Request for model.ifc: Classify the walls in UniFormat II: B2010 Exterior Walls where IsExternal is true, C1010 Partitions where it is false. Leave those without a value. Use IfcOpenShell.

First a look at what the model holds.

```python
import ifcopenshell
import ifcopenshell.util.element

model = ifcopenshell.open("model.ifc")
print(model.schema)
print("classifications:", [c.Name for c in model.by_type("IfcClassification")])
values = [ifcopenshell.util.element.get_pset(e, "Pset_WallCommon", "IsExternal") for e in model.by_type("IfcWall")]
for value in (True, False, None):
    print("IsExternal", value, values.count(value))
```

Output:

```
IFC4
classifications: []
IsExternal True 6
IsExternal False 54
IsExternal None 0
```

```python
import ifcopenshell
import ifcopenshell.api.classification
import ifcopenshell.util.element

model = ifcopenshell.open("model.ifc")

system = ifcopenshell.api.classification.add_classification(model, classification="UniFormat II")

walls = model.by_type("IfcWall")
external = {e: ifcopenshell.util.element.get_pset(e, "Pset_WallCommon", "IsExternal") for e in walls}
for flag, code, name in ((True, "B2010", "Exterior Walls"), (False, "C1010", "Partitions")):
    products = [e for e in walls if external[e] is flag]
    ifcopenshell.api.classification.add_reference(
        model, products=products, classification=system, identification=code, name=name
    )
    print(code, len(products))

model.write("model_edited.ifc")
```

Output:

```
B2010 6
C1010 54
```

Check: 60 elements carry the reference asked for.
